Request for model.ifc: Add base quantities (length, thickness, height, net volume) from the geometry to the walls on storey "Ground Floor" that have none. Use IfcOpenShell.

First a look at what the model holds.

```python
import ifcopenshell
import ifcopenshell.util.element
import ifcopenshell.util.unit

model = ifcopenshell.open("model.ifc")
print(model.schema)
for unit_type in ("LENGTHUNIT", "AREAUNIT", "VOLUMEUNIT"):
    print(unit_type, ifcopenshell.util.unit.calculate_unit_scale(model, unit_type))
storey = next(s for s in model.by_type("IfcBuildingStorey") if s.Name == "Ground Floor")
walls = [e for e in ifcopenshell.util.element.get_decomposition(storey) if e.is_a("IfcWall")]
for e in sorted(walls, key=lambda e: e.id()):
    print(e.id(), e.is_a(), e.Name, list(ifcopenshell.util.element.get_psets(e, qtos_only=True)), sep=" | ")
```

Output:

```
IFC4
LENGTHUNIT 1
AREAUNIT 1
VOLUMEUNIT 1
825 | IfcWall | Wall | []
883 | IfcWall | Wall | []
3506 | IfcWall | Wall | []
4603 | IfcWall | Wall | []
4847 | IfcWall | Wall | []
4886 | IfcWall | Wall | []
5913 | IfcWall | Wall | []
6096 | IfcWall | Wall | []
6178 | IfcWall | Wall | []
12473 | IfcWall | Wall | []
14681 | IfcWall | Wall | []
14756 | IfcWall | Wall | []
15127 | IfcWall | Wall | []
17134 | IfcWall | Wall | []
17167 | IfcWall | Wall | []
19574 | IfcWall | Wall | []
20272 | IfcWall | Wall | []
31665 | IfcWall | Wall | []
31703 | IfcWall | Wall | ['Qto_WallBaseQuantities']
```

```python
import ifcopenshell
import ifcopenshell.api.pset
import ifcopenshell.geom
import ifcopenshell.util.element
import ifcopenshell.util.shape
import ifcopenshell.util.unit

model = ifcopenshell.open("model.ifc")
unit_scale = ifcopenshell.util.unit.calculate_unit_scale(model)
volume_scale = ifcopenshell.util.unit.calculate_unit_scale(model, "VOLUMEUNIT")
settings = ifcopenshell.geom.settings()

storey = next(s for s in model.by_type("IfcBuildingStorey") if s.Name == "Ground Floor")
walls = [e for e in ifcopenshell.util.element.get_decomposition(storey) if e.is_a("IfcWall")]

for e in sorted(walls, key=lambda e: e.id()):
    if ifcopenshell.util.element.get_psets(e, qtos_only=True, should_inherit=False):
        continue
    # Geometry comes back in metres, in the element's own axes.
    shape = ifcopenshell.geom.create_shape(settings, e)
    values = {
        "Length": ifcopenshell.util.shape.get_x(shape.geometry) / unit_scale,
        "Width": ifcopenshell.util.shape.get_y(shape.geometry) / unit_scale,
        "Height": ifcopenshell.util.shape.get_z(shape.geometry) / unit_scale,
        "NetVolume": ifcopenshell.util.shape.get_volume(shape.geometry) / volume_scale,
    }
    qto = ifcopenshell.api.pset.add_qto(model, product=e, name="Qto_WallBaseQuantities")
    ifcopenshell.api.pset.edit_qto(model, qto=qto, properties=values)
    print(e.id(), {k: round(v, 3) for k, v in values.items()})

model.write("model-out.ifc")
```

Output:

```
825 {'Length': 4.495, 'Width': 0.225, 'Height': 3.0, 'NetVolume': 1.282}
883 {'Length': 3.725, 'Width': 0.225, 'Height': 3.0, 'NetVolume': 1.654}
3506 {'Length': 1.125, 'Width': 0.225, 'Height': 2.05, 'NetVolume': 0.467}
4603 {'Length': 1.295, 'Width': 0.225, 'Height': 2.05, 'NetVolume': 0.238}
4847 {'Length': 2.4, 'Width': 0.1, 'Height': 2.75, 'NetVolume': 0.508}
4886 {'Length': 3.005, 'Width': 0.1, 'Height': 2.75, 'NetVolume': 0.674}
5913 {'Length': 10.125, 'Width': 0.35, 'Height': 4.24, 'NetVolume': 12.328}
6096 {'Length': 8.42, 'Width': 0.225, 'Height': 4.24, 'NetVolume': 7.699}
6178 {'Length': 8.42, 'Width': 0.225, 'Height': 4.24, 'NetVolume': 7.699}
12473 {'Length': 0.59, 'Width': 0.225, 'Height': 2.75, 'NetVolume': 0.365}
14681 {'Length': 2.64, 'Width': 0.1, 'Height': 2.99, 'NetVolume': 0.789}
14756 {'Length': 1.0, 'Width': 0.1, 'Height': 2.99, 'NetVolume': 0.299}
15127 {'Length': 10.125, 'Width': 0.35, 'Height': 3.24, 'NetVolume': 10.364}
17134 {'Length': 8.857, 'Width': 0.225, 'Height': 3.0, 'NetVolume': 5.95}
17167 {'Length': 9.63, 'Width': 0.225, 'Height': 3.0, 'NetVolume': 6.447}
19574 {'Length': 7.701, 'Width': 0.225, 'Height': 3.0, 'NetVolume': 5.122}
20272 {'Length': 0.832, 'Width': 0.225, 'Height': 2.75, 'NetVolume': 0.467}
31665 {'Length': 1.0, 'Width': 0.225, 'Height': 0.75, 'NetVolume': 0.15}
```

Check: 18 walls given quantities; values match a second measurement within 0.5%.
